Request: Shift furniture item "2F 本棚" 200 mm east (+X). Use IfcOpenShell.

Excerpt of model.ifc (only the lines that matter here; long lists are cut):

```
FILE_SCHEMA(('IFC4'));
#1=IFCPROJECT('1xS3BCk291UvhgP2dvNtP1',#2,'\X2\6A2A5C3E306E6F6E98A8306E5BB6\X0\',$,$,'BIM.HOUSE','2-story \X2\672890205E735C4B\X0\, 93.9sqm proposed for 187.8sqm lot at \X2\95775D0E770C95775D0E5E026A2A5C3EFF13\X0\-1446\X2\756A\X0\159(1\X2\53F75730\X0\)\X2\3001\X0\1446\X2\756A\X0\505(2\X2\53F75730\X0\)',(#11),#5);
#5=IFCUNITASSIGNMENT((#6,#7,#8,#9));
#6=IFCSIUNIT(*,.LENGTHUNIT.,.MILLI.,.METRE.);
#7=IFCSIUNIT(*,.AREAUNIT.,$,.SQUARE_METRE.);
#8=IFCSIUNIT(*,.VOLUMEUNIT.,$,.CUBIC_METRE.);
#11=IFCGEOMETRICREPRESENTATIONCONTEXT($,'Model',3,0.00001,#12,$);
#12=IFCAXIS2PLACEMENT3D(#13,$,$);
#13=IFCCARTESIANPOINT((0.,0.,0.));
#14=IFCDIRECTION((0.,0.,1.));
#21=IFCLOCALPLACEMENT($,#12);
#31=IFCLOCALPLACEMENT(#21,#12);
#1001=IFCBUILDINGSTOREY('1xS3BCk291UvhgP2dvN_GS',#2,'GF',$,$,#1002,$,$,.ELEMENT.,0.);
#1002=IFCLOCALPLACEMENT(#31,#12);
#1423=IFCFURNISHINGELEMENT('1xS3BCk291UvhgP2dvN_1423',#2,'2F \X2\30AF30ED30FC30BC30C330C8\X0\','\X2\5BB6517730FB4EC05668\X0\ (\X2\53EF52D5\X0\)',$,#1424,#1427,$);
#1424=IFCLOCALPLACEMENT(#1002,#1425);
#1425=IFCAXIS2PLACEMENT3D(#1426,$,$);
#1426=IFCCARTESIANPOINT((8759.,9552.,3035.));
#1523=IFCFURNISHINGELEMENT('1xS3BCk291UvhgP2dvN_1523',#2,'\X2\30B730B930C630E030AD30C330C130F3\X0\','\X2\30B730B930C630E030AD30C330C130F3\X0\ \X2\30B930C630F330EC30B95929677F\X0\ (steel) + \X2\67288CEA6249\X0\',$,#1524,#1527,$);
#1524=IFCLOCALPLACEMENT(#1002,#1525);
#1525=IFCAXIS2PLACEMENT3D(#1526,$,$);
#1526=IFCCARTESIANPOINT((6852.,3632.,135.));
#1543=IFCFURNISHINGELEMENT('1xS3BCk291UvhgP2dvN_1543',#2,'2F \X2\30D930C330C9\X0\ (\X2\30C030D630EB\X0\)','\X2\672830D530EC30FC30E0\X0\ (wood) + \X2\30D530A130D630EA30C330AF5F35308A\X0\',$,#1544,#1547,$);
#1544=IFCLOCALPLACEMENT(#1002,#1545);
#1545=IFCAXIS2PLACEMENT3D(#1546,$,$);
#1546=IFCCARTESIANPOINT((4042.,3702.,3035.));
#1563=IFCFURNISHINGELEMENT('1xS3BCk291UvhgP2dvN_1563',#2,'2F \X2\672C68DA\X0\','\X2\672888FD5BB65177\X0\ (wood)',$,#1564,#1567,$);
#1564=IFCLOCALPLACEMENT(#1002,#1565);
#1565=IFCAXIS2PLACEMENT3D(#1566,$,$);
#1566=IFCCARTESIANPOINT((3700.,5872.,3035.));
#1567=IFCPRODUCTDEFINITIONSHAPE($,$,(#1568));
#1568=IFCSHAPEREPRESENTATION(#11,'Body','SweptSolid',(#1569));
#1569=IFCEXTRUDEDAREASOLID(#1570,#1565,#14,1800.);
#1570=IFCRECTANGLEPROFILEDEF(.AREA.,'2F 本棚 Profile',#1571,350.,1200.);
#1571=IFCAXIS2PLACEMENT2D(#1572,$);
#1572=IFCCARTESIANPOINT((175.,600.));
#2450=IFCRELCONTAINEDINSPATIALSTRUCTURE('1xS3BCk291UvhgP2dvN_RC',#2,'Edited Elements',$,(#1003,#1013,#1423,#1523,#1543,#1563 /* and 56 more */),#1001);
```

```python
import ifcopenshell
import ifcopenshell.api.geometry
import ifcopenshell.util.placement
import ifcopenshell.util.unit

model = ifcopenshell.open("model.ifc")
unit_scale = ifcopenshell.util.unit.calculate_unit_scale(model)

item = model.by_guid("1xS3BCk291UvhgP2dvN_1563")
matrix = ifcopenshell.util.placement.get_local_placement(item.ObjectPlacement)
matrix[0, 3] += 0.2 / unit_scale
ifcopenshell.api.geometry.edit_object_placement(model, product=item, matrix=matrix, is_si=False)

print(ifcopenshell.util.placement.get_local_placement(item.ObjectPlacement).round(3) + 0.0)

model.write("model_edited.ifc")
```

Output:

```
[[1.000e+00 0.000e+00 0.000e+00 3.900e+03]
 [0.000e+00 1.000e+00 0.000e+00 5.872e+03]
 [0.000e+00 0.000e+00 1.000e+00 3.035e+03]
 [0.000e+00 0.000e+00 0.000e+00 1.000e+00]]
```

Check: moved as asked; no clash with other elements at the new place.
